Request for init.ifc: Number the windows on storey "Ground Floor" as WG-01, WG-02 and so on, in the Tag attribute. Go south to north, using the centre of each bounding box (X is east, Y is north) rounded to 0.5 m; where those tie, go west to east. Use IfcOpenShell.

First a look at what the model holds.

```python
import ifcopenshell
import ifcopenshell.util.element
import ifcopenshell.util.placement

model = ifcopenshell.open("init.ifc")
print(model.schema)
storey = next(s for s in model.by_type("IfcBuildingStorey") if s.Name == "Ground Floor")
windows = [e for e in ifcopenshell.util.element.get_decomposition(storey) if e.is_a("IfcWindow")]
for e in sorted(windows, key=lambda e: e.id()):
    origin = ifcopenshell.util.placement.get_local_placement(e.ObjectPlacement)[:3, 3]
    print(e.id(), e.Tag, e.Name, origin.round(2) + 0.0, sep=" | ")
```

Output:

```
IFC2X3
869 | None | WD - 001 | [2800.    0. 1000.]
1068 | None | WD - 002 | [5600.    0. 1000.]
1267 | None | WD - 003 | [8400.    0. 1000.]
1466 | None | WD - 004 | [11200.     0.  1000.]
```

```python
import ifcopenshell
import ifcopenshell.geom
import ifcopenshell.util.element
import ifcopenshell.util.shape

model = ifcopenshell.open("init.ifc")
settings = ifcopenshell.geom.settings()
settings.set("use-world-coords", True)


def centre(element):
    shape = ifcopenshell.geom.create_shape(settings, element)
    return ifcopenshell.util.shape.get_bbox_centroid(shape.geometry)


storey = next(s for s in model.by_type("IfcBuildingStorey") if s.Name == "Ground Floor")
windows = [e for e in ifcopenshell.util.element.get_decomposition(storey) if e.is_a("IfcWindow")]

# Insertion points can sit at a corner or the storey origin, so sort by the geometry (in metres).
centres = {e: centre(e) for e in windows}
windows.sort(key=lambda e: (round(centres[e][1] / 0.5), centres[e][0]))

for i, e in enumerate(windows, start=1):
    number = f"WG-{i:02d}"
    e.Tag = number
    print(e.id(), number)

model.write("init_rev.ifc")
```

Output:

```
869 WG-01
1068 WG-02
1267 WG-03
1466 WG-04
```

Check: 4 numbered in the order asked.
